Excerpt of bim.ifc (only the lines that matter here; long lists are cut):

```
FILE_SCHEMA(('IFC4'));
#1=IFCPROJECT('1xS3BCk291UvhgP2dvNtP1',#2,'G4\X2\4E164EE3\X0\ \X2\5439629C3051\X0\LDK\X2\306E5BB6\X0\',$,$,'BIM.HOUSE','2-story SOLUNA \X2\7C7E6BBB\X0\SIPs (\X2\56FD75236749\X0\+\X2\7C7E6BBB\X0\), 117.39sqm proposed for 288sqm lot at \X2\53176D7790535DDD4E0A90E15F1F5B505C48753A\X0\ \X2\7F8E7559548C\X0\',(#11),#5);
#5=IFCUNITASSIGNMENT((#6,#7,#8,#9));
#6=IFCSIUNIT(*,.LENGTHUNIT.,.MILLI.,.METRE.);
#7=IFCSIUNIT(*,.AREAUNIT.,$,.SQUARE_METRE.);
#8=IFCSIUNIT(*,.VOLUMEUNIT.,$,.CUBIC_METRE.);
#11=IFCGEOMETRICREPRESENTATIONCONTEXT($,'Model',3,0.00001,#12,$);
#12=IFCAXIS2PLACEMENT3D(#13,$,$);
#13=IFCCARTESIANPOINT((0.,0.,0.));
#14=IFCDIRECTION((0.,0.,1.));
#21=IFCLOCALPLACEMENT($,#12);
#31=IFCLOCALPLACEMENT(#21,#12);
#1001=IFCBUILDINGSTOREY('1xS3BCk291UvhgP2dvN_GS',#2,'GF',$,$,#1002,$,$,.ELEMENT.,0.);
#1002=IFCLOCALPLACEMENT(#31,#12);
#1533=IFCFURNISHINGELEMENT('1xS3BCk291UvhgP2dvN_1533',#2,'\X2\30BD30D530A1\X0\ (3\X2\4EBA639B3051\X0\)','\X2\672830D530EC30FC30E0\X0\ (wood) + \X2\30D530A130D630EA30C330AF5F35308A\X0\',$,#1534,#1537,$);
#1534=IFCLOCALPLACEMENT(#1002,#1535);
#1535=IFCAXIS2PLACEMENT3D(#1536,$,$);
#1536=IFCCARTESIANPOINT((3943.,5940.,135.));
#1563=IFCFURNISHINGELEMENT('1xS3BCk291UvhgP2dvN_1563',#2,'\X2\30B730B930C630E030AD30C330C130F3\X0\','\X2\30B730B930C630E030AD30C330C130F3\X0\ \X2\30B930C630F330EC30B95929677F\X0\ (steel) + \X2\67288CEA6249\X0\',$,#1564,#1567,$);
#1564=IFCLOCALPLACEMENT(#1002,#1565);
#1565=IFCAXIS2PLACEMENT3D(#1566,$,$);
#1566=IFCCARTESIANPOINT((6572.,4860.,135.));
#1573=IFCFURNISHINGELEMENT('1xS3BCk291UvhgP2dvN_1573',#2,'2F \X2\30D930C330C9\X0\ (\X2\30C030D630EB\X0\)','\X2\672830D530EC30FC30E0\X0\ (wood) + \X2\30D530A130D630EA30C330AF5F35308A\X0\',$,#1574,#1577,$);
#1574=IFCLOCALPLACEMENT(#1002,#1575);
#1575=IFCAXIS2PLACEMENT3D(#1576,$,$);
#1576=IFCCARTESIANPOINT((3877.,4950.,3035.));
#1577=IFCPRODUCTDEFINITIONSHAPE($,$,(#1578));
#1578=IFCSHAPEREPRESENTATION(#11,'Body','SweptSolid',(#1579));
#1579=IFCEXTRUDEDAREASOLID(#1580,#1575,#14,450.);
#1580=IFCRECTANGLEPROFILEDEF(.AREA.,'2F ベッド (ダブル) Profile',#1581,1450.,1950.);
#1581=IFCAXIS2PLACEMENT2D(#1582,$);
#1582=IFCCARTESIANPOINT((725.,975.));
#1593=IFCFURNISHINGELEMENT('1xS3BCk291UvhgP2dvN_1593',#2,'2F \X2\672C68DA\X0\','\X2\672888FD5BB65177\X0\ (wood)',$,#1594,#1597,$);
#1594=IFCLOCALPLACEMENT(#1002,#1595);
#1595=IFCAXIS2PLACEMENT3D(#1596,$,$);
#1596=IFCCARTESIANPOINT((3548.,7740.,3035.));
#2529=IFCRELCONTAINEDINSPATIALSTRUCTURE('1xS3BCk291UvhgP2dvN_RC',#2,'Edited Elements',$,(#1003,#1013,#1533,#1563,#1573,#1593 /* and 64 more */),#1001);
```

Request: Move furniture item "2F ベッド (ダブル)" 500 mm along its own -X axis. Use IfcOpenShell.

```python
import ifcopenshell
import ifcopenshell.api.geometry
import ifcopenshell.util.placement
import ifcopenshell.util.unit

model = ifcopenshell.open("bim.ifc")
unit_scale = ifcopenshell.util.unit.calculate_unit_scale(model)

item = model.by_id(1573)
matrix = ifcopenshell.util.placement.get_local_placement(item.ObjectPlacement)
matrix[:3, 3] -= matrix[:3, 0] * 0.5 / unit_scale
ifcopenshell.api.geometry.edit_object_placement(model, product=item, matrix=matrix, is_si=False)

print(ifcopenshell.util.placement.get_local_placement(item.ObjectPlacement).round(3) + 0.0)

model.write("bim_v2.ifc")
```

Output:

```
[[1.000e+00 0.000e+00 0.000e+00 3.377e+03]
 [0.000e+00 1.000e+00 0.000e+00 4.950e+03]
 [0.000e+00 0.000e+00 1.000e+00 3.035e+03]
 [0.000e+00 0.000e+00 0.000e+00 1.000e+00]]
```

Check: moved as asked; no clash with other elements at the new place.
